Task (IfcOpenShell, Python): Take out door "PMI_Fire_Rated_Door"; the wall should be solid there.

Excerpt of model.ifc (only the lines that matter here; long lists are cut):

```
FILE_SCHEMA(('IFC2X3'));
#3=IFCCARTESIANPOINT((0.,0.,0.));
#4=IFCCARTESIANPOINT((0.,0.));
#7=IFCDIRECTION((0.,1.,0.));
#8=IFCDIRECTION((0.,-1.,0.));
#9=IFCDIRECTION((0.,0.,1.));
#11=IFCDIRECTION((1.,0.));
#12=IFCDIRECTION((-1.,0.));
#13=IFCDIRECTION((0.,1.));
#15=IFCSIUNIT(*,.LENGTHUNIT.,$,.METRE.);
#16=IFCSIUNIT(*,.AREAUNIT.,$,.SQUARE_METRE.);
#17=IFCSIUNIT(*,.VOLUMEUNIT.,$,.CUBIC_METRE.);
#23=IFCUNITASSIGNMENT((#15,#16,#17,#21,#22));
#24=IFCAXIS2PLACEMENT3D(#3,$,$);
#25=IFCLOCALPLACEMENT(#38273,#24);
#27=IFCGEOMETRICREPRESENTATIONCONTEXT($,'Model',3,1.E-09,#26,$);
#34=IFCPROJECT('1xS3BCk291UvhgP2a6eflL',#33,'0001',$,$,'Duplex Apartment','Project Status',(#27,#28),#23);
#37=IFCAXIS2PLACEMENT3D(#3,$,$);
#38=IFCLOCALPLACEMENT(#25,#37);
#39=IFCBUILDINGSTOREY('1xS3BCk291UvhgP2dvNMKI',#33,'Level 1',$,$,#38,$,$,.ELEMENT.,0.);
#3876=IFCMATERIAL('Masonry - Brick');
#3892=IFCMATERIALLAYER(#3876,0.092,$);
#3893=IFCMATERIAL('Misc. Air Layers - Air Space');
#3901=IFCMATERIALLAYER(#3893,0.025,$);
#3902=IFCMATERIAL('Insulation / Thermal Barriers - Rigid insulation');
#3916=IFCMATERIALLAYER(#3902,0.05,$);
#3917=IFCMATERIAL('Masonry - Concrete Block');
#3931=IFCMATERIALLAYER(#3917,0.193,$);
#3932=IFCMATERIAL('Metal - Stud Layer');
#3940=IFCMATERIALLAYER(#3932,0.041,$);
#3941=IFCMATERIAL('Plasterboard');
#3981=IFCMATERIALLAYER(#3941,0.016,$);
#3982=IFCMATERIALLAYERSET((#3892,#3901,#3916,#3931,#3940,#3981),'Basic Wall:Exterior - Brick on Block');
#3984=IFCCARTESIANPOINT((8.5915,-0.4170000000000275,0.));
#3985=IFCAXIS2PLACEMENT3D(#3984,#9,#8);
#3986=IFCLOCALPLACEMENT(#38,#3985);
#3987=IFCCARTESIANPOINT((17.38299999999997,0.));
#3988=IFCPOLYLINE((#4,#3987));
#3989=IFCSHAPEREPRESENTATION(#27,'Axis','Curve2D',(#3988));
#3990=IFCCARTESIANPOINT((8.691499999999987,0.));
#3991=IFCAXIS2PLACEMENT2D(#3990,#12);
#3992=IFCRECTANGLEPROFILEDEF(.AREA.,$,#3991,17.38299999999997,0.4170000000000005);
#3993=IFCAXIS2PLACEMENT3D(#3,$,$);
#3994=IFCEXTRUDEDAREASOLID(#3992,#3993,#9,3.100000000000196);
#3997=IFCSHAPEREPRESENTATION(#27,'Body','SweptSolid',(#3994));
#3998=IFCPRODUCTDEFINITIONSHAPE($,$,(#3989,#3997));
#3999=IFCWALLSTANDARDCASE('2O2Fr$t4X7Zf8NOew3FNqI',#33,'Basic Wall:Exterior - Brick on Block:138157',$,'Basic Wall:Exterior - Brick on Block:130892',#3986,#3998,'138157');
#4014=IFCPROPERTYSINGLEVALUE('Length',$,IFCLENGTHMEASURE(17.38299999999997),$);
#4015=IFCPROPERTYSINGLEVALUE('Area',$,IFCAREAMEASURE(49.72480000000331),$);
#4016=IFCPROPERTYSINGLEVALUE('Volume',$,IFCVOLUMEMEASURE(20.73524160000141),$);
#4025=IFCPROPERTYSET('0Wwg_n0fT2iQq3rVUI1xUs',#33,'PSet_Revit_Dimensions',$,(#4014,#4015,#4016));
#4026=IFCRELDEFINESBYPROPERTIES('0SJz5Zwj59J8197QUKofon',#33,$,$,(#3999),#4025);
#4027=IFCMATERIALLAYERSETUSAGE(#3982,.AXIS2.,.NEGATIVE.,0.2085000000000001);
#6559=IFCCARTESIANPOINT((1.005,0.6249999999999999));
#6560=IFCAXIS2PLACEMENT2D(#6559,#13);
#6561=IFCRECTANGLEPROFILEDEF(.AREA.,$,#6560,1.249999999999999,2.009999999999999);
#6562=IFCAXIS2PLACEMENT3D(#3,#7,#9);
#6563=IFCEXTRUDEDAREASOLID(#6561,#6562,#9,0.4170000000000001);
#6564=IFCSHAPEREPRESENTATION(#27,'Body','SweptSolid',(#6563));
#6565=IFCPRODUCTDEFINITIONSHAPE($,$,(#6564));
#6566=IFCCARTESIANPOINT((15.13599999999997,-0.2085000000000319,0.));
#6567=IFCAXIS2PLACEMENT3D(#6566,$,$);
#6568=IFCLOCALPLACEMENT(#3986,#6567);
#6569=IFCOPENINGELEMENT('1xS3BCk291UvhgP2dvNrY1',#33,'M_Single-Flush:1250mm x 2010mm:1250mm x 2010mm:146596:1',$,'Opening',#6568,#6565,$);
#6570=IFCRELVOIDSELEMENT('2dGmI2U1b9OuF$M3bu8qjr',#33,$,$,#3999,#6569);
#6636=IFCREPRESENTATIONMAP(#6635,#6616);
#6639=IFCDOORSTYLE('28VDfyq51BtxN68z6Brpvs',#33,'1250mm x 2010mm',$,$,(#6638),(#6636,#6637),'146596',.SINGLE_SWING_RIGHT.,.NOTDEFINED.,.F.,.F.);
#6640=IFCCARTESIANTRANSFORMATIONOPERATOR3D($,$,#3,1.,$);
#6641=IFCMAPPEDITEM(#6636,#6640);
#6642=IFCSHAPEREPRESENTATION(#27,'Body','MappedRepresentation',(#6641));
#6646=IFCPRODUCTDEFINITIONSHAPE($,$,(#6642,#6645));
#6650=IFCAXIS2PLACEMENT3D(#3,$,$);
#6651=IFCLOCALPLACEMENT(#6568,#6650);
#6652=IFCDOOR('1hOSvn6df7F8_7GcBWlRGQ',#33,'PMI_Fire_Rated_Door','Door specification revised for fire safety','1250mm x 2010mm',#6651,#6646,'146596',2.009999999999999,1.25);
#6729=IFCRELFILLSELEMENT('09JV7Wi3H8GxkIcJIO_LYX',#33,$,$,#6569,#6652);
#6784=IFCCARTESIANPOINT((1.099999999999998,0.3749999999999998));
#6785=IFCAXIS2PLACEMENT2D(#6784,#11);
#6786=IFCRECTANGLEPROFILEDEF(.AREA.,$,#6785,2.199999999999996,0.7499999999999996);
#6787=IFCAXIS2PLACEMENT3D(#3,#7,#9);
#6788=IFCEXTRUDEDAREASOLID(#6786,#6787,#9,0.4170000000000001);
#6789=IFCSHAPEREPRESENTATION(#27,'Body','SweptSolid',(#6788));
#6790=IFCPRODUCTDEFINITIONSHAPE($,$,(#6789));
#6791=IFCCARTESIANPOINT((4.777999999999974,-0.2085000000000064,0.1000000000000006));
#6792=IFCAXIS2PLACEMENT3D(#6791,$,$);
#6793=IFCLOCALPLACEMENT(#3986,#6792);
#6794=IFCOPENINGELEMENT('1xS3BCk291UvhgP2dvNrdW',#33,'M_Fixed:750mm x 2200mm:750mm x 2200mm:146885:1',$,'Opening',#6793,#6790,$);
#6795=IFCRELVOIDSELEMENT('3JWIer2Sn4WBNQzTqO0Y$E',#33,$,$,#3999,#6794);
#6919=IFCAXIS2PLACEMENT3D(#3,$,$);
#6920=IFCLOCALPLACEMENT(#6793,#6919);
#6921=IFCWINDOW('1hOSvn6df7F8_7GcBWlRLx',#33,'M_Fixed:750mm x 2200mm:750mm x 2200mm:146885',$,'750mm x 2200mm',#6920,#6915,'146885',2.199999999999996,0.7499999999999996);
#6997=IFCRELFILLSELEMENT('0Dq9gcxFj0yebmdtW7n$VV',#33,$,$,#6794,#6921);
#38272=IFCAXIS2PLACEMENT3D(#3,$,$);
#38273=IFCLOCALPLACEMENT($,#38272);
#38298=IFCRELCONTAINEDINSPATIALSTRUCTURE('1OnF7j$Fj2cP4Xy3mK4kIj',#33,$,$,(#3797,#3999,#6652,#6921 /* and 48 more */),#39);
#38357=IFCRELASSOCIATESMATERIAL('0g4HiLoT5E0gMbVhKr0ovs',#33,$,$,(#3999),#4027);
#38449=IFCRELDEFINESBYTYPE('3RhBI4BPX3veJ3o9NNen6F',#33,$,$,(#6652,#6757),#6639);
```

```python
import ifcopenshell
import ifcopenshell.api.feature
import ifcopenshell.api.pset
import ifcopenshell.api.root
import ifcopenshell.geom
import ifcopenshell.util.element
import ifcopenshell.util.shape
import ifcopenshell.util.unit

model = ifcopenshell.open("model.ifc")
area_scale = ifcopenshell.util.unit.calculate_unit_scale(model, "AREAUNIT")
volume_scale = ifcopenshell.util.unit.calculate_unit_scale(model, "VOLUMEUNIT")
settings = ifcopenshell.geom.settings()


def volume(element):
    """Net volume in cubic metres, openings subtracted."""
    shape = ifcopenshell.geom.create_shape(settings, element)
    return ifcopenshell.util.shape.get_volume(shape.geometry)


door = model.by_guid("1hOSvn6df7F8_7GcBWlRGQ")
opening = door.FillsVoids[0].RelatingOpeningElement
wall = opening.VoidsElements[0].RelatingBuildingElement
before = volume(wall)

ifcopenshell.api.root.remove_product(model, product=door)
ifcopenshell.api.feature.remove_feature(model, feature=opening)

after = volume(wall)
thickness = 0.417  # wall thickness in metres

# Update the wall's stored quantities.
pset = model.by_id(ifcopenshell.util.element.get_pset(wall, "PSet_Revit_Dimensions", should_inherit=False)["id"])
ifcopenshell.api.pset.edit_pset(model, pset=pset, properties={
    "Area": model.create_entity("IfcAreaMeasure", after / thickness / area_scale),
    "Volume": model.create_entity("IfcVolumeMeasure", after / volume_scale),
})

print(f"wall volume {before:.3f} -> {after:.3f} m3")

model.write("model-out.ifc")
```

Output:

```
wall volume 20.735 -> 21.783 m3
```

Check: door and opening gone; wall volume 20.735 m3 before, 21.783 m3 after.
